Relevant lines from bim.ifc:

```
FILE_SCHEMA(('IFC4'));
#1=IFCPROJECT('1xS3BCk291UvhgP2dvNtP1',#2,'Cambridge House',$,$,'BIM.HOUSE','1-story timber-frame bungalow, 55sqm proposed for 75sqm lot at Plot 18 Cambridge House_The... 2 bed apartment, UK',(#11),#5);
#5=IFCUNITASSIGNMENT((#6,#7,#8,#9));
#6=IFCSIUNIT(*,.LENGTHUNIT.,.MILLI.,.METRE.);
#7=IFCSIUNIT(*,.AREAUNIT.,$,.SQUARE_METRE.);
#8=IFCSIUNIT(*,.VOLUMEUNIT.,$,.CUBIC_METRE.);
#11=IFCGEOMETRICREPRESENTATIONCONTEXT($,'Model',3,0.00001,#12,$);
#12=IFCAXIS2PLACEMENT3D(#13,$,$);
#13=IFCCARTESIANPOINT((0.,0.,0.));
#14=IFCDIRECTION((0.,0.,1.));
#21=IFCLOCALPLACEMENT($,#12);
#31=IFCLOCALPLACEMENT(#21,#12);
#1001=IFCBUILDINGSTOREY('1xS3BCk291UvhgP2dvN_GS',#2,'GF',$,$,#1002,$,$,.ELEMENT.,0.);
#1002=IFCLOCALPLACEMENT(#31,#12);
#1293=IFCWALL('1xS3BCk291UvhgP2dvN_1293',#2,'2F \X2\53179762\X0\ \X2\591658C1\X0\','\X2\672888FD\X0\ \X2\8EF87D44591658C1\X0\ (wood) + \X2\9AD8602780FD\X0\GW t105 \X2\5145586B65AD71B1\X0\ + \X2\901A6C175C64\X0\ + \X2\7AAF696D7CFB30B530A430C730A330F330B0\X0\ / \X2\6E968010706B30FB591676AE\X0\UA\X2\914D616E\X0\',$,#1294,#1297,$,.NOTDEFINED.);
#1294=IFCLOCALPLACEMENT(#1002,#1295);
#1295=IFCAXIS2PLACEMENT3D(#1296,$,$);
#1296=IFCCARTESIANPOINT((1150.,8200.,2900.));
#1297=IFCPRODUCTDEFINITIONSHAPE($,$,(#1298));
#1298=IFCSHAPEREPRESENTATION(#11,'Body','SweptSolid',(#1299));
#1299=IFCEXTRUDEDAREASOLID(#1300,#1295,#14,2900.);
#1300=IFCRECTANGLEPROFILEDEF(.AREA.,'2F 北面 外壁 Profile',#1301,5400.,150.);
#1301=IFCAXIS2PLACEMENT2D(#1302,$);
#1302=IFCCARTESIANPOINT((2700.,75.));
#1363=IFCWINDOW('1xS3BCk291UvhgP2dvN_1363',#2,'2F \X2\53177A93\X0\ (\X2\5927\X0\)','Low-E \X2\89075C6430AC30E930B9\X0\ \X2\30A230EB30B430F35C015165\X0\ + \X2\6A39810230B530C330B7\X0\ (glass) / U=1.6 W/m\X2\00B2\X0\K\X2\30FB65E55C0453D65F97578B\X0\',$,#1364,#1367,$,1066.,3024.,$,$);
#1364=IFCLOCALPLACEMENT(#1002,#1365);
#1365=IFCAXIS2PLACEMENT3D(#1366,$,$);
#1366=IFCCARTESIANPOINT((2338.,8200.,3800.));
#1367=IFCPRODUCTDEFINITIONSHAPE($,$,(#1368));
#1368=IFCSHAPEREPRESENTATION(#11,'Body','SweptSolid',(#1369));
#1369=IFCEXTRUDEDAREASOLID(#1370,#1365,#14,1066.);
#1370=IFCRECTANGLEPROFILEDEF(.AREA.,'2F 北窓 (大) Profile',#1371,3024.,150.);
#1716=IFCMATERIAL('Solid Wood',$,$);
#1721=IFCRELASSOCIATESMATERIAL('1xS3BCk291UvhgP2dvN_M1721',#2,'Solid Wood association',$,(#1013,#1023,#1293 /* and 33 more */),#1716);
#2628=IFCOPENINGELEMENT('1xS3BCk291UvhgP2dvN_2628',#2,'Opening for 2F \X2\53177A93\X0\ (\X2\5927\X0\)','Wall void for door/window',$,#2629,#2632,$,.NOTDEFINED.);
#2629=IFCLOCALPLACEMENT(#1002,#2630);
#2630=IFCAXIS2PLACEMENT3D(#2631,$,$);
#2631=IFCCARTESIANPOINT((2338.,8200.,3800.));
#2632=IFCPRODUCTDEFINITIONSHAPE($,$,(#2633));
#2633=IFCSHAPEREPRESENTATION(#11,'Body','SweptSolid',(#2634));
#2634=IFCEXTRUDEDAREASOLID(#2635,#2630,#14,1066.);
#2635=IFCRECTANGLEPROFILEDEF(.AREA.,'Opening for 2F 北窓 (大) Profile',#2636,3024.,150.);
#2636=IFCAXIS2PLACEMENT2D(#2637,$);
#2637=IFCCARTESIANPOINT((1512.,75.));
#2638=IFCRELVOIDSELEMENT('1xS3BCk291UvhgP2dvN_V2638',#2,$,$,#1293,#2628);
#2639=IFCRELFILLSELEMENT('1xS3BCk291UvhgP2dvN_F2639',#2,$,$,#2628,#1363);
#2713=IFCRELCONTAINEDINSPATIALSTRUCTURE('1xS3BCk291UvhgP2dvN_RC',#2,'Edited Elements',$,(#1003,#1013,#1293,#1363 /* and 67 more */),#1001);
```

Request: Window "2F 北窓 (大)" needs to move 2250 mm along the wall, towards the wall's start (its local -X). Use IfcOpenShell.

```python
import ifcopenshell
import ifcopenshell.api.geometry
import ifcopenshell.util.placement

model = ifcopenshell.open("bim.ifc")

window = model.by_guid("1xS3BCk291UvhgP2dvN_1363")
opening = window.FillsVoids[0].RelatingOpeningElement
wall = opening.VoidsElements[0].RelatingBuildingElement

wall_matrix = ifcopenshell.util.placement.get_local_placement(wall.ObjectPlacement)
shift = wall_matrix[:3, 0] * -2250.0
before = ifcopenshell.util.placement.get_local_placement(window.ObjectPlacement)[:3, 3].copy()

# The window is not placed relative to its opening, so move both.
for product in (opening, window):
    matrix = ifcopenshell.util.placement.get_local_placement(product.ObjectPlacement)
    matrix[:3, 3] += shift
    ifcopenshell.api.geometry.edit_object_placement(model, product=product, matrix=matrix, is_si=False)

after = ifcopenshell.util.placement.get_local_placement(window.ObjectPlacement)[:3, 3]
print("window moved by", (after - before).round(3) + 0.0)

model.write("bim-out.ifc")
```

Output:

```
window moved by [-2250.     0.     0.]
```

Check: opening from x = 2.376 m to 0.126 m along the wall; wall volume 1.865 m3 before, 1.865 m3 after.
